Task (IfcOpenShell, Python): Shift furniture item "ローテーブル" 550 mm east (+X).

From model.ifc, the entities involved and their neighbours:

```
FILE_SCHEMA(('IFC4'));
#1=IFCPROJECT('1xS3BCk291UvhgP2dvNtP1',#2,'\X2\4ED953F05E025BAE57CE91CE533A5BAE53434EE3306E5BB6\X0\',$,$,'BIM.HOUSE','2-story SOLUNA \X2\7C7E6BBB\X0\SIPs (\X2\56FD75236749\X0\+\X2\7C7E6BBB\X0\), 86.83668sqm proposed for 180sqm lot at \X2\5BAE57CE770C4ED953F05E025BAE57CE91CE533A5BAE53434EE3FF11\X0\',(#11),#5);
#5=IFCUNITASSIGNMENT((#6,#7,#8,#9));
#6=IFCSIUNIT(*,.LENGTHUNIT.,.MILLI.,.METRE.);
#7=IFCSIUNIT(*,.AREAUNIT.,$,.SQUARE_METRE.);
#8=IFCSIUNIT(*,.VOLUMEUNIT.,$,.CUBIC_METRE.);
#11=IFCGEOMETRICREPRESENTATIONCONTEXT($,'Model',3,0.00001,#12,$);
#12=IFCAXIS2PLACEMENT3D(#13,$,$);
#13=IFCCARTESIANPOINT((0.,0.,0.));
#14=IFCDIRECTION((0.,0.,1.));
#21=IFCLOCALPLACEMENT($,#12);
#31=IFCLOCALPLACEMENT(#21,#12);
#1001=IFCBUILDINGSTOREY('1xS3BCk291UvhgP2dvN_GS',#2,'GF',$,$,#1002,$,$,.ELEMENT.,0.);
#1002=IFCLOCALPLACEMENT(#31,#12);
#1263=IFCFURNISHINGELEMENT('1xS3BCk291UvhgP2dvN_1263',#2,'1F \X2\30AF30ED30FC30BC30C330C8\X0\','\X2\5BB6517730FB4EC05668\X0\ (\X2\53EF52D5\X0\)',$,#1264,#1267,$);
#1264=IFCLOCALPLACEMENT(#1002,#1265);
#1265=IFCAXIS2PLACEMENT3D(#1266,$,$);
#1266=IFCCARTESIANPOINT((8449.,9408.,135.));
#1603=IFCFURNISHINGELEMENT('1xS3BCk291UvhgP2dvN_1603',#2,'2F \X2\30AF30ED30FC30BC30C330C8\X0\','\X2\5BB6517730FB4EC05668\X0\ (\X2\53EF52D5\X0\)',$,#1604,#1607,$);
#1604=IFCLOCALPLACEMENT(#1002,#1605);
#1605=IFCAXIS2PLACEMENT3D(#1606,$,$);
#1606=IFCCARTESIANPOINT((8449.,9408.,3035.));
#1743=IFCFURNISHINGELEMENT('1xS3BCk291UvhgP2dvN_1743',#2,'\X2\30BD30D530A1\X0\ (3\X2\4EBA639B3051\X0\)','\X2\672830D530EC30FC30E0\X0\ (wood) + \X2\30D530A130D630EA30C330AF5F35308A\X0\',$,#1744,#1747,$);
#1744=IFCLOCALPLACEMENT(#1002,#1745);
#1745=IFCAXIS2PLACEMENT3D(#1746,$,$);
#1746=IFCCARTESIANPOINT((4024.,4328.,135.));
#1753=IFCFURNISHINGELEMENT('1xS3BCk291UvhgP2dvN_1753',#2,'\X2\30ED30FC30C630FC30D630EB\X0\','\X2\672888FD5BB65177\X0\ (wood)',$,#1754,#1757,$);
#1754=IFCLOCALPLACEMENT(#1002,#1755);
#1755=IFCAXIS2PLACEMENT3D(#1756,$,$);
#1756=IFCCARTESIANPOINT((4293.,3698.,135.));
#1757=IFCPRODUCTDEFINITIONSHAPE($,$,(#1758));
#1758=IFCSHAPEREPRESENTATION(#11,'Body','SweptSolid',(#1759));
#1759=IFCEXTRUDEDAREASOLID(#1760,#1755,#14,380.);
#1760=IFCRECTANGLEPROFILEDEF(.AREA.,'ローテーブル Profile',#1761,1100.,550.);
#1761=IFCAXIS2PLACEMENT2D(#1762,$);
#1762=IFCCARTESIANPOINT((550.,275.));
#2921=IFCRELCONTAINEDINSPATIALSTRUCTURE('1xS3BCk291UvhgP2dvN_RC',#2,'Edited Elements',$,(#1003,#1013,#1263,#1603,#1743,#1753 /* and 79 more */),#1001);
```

```python
import ifcopenshell
import ifcopenshell.api.geometry
import ifcopenshell.util.placement
import ifcopenshell.util.unit

model = ifcopenshell.open("model.ifc")
unit_scale = ifcopenshell.util.unit.calculate_unit_scale(model)

item = model.by_id(1753)
matrix = ifcopenshell.util.placement.get_local_placement(item.ObjectPlacement)
matrix[0, 3] += 0.55 / unit_scale
ifcopenshell.api.geometry.edit_object_placement(model, product=item, matrix=matrix, is_si=False)

print(ifcopenshell.util.placement.get_local_placement(item.ObjectPlacement).round(3) + 0.0)

model.write("model_v2.ifc")
```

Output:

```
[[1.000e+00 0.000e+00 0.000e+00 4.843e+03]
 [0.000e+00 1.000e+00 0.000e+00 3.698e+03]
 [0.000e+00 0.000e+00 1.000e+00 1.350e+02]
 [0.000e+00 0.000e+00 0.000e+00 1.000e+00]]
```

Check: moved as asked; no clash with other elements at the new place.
